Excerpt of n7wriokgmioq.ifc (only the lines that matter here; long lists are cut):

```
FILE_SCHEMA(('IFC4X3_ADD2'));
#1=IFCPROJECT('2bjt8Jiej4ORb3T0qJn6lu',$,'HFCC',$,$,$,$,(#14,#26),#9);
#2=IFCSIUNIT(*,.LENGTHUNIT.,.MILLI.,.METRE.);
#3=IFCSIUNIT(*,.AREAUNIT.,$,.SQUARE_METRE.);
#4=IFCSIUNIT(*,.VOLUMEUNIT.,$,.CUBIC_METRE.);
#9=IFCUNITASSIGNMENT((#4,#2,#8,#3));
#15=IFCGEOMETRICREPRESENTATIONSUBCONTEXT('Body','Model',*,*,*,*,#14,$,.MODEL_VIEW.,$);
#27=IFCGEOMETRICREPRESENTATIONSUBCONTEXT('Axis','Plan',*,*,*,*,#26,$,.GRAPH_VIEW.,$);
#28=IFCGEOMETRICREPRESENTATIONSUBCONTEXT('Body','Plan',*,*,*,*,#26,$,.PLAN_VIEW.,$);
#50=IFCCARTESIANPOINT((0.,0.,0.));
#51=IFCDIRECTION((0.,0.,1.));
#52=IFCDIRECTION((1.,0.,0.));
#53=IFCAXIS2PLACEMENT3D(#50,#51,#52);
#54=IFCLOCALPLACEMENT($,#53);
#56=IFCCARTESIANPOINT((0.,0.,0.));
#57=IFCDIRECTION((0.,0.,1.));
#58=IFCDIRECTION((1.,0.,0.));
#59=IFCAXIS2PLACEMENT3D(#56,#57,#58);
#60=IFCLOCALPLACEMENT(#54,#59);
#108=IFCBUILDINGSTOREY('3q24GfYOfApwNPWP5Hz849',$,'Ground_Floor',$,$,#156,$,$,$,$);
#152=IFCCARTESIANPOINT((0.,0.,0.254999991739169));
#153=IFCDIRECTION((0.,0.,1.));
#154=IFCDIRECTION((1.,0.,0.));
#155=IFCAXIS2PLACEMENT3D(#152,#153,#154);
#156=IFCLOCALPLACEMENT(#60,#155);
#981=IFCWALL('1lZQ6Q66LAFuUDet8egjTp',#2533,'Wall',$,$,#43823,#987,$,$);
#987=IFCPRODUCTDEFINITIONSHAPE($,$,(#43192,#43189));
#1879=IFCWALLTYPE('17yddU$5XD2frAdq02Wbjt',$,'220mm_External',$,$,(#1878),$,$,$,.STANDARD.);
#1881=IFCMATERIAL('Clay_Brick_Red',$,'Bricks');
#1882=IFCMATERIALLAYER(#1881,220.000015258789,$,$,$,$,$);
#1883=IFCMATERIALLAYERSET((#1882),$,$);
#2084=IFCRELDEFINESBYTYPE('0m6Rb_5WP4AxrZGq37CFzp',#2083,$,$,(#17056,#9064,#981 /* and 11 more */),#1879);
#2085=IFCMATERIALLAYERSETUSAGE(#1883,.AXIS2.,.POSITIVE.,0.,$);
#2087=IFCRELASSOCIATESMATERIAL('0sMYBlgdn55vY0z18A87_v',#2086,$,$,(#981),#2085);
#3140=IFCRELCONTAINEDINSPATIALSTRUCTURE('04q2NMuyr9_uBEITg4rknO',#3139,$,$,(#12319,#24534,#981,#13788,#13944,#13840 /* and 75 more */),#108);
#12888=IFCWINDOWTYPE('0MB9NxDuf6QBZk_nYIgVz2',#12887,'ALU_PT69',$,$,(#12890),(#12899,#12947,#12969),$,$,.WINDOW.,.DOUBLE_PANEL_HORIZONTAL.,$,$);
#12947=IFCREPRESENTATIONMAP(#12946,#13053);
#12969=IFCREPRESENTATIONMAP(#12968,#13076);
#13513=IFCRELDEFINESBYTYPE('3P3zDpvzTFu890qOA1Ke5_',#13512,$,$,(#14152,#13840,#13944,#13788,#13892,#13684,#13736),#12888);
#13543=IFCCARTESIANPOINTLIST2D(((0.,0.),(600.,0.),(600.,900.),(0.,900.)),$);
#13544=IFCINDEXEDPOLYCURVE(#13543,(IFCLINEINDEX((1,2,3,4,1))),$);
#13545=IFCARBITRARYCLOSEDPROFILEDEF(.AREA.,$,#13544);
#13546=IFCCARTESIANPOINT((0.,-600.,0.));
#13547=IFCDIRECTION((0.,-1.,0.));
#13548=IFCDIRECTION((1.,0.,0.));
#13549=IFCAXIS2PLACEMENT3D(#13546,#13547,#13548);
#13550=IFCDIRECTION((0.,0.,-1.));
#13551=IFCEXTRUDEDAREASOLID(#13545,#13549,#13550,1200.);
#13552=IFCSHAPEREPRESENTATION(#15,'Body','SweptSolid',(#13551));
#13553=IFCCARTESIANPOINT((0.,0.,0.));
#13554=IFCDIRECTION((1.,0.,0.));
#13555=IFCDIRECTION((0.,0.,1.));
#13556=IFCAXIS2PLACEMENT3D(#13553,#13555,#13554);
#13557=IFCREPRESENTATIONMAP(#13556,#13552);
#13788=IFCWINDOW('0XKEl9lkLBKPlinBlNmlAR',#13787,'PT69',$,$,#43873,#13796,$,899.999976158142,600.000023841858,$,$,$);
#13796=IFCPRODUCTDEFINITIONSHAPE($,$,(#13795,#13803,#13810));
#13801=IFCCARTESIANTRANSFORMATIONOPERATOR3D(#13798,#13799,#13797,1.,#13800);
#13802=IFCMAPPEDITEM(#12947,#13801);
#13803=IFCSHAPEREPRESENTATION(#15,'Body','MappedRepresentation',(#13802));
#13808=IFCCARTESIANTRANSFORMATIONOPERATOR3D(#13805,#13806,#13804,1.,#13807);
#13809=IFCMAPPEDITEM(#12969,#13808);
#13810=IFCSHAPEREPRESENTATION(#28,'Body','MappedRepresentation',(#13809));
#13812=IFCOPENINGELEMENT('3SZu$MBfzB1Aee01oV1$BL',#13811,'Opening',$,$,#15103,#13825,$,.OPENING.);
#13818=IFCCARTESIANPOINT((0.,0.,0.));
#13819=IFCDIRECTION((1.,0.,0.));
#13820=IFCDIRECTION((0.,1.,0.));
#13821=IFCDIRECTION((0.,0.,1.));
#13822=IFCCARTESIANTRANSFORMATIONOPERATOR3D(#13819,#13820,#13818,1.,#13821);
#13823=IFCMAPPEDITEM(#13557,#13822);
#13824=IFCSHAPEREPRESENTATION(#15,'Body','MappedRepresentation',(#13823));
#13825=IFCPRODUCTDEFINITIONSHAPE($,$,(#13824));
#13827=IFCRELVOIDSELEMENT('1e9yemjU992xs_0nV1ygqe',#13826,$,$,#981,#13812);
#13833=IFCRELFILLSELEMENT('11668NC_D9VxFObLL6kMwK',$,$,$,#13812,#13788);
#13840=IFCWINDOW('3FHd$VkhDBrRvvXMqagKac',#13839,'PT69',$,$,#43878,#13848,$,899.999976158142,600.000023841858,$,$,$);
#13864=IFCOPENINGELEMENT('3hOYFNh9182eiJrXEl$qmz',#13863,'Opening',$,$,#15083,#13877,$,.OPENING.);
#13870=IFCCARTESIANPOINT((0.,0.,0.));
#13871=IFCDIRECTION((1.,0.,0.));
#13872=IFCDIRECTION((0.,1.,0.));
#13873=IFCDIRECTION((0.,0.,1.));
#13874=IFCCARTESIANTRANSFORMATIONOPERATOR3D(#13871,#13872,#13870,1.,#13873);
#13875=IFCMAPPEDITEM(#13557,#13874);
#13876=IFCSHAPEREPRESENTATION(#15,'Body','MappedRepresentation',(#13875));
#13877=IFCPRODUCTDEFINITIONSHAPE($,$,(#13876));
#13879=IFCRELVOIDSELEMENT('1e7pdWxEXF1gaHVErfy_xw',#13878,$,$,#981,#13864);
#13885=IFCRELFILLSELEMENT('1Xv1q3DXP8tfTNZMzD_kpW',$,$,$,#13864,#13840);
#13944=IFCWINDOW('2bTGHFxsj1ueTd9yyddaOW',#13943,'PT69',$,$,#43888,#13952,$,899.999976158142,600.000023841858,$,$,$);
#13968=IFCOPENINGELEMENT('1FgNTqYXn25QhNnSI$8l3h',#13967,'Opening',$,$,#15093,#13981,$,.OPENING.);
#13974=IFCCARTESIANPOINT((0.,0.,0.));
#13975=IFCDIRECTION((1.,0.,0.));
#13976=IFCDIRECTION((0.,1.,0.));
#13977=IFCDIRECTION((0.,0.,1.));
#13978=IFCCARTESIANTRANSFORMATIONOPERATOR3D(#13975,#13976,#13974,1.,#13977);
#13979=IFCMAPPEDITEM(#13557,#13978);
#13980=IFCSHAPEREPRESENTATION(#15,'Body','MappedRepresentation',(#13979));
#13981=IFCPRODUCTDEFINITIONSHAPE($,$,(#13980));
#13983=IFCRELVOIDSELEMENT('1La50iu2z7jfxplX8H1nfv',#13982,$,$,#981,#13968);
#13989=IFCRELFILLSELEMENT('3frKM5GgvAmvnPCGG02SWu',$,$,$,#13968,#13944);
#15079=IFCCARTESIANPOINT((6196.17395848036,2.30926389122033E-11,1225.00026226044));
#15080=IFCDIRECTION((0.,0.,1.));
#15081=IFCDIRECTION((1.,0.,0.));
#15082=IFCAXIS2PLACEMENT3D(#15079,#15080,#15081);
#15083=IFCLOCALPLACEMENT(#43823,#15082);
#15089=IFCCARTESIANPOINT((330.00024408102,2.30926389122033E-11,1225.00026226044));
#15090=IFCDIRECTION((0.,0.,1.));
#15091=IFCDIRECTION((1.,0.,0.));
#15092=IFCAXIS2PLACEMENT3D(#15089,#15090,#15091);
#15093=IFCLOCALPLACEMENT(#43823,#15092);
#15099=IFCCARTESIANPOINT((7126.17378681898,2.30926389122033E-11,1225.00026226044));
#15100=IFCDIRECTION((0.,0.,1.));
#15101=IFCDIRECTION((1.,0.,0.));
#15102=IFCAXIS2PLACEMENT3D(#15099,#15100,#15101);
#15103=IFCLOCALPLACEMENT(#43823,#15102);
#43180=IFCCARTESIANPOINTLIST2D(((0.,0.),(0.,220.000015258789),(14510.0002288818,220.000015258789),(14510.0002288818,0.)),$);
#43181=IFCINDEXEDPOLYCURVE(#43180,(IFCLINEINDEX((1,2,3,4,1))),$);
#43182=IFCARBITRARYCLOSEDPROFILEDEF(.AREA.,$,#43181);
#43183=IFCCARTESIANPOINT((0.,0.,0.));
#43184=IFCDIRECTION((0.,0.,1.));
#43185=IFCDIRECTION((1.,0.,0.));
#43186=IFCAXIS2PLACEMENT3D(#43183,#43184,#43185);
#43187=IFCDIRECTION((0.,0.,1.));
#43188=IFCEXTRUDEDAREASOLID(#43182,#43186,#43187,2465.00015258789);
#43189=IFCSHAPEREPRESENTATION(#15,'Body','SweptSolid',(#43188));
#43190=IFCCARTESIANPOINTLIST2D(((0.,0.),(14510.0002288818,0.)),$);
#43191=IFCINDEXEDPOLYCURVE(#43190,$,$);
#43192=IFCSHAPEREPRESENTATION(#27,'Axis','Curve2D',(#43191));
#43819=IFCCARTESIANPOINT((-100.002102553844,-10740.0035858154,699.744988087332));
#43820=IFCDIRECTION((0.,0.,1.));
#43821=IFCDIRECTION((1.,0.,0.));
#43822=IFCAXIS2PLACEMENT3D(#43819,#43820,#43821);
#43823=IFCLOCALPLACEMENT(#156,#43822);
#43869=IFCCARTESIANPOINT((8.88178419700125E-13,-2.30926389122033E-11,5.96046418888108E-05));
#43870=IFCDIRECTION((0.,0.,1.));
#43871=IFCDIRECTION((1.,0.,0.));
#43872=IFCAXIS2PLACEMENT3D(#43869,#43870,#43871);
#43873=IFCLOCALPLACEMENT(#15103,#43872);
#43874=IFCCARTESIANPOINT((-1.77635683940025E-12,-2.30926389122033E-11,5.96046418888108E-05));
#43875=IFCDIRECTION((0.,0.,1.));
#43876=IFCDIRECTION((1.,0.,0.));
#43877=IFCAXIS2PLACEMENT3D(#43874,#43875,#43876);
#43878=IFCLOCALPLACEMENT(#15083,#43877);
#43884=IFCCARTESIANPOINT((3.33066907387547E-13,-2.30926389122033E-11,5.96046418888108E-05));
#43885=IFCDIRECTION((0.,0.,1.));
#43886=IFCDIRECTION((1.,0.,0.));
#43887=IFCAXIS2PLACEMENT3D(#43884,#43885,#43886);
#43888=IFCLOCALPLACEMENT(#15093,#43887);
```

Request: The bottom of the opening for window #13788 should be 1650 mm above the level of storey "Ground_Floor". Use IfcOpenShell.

```python
import numpy as np
import ifcopenshell
import ifcopenshell.api.geometry
import ifcopenshell.geom
import ifcopenshell.util.element
import ifcopenshell.util.placement
import ifcopenshell.util.shape
import ifcopenshell.util.unit

model = ifcopenshell.open("n7wriokgmioq.ifc")
unit_scale = ifcopenshell.util.unit.calculate_unit_scale(model)

window = model.by_id(13788)
opening = window.FillsVoids[0].RelatingOpeningElement
storey = ifcopenshell.util.element.get_container(window, ifc_class="IfcBuildingStorey")
level = ifcopenshell.util.placement.get_local_placement(storey.ObjectPlacement)[2, 3]

# The opening's origin need not be at the sill, so measure its lowest point.
shape = ifcopenshell.geom.create_shape(ifcopenshell.geom.settings(), opening)
bottom = ifcopenshell.util.shape.get_shape_bottom_elevation(shape, shape.geometry) / unit_scale
dz = level + 1.65 / unit_scale - bottom

shift = np.array([0.0, 0.0, dz])
# The window is placed relative to its opening, so it follows when the opening moves.
matrix = ifcopenshell.util.placement.get_local_placement(opening.ObjectPlacement)
matrix[:3, 3] += shift
ifcopenshell.api.geometry.edit_object_placement(
    model, product=opening, matrix=matrix, is_si=False, should_transform_children=True
)

print(f"moved by {dz * unit_scale:+.3f} m")

model.write("n7wriokgmioq_rev.ifc")
```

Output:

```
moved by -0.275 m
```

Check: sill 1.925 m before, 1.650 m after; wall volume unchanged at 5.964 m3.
